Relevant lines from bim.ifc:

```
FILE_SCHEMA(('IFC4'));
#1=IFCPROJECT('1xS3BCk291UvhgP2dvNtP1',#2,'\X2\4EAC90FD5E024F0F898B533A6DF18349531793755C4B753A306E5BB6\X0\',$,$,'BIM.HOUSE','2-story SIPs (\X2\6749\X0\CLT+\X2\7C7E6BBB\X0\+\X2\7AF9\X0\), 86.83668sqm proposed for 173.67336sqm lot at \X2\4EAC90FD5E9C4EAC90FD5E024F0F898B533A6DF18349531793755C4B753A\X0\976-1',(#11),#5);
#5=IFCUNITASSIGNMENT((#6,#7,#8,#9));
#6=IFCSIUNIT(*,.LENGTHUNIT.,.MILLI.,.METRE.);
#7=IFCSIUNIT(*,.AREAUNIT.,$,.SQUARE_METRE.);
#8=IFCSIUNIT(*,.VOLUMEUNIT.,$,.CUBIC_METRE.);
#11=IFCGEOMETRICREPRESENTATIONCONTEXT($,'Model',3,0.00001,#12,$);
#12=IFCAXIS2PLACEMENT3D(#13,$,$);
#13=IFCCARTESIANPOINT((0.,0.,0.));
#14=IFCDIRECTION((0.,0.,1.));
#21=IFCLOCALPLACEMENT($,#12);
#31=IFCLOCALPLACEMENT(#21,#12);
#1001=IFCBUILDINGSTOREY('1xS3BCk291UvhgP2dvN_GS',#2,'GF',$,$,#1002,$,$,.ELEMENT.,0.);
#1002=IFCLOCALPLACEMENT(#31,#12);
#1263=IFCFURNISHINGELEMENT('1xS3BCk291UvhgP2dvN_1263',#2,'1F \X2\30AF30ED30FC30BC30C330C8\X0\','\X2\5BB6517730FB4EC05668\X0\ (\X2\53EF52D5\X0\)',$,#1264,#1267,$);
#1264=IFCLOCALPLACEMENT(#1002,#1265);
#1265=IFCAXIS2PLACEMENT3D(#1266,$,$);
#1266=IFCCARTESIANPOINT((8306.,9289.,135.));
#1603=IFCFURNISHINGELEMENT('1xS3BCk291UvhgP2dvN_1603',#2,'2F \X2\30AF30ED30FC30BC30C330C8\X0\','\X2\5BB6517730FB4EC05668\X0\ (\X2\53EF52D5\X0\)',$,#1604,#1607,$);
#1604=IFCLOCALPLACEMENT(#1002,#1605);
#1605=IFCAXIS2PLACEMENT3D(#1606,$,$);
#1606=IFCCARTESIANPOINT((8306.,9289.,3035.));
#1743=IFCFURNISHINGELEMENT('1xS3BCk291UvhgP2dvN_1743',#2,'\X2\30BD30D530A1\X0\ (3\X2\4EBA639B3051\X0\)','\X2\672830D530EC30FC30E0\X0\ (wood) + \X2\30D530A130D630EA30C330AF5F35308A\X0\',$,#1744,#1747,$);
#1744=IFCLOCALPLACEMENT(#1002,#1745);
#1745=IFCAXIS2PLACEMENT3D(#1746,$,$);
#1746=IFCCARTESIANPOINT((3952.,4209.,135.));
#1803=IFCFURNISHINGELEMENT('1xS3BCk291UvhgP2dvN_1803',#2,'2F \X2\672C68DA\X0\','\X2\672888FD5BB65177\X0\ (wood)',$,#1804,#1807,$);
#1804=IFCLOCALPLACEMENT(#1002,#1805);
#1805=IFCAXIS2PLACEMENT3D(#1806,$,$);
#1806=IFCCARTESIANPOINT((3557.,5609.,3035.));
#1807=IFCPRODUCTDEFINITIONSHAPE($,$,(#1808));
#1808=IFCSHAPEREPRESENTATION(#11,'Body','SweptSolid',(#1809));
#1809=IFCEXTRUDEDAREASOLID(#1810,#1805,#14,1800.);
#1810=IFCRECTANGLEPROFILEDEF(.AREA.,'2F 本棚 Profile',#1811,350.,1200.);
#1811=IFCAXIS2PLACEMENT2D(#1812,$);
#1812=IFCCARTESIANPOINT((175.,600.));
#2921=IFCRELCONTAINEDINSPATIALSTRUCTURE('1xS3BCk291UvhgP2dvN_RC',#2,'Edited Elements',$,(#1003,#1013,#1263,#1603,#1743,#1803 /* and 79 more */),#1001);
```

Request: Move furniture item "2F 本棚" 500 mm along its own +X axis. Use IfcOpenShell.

```python
import ifcopenshell
import ifcopenshell.api.geometry
import ifcopenshell.util.placement

model = ifcopenshell.open("bim.ifc")

item = model.by_guid("1xS3BCk291UvhgP2dvN_1803")
matrix = ifcopenshell.util.placement.get_local_placement(item.ObjectPlacement)
matrix[:3, 3] += matrix[:3, 0] * 500.0
ifcopenshell.api.geometry.edit_object_placement(model, product=item, matrix=matrix, is_si=False)

print(ifcopenshell.util.placement.get_local_placement(item.ObjectPlacement).round(3) + 0.0)

model.write("bim_edited.ifc")
```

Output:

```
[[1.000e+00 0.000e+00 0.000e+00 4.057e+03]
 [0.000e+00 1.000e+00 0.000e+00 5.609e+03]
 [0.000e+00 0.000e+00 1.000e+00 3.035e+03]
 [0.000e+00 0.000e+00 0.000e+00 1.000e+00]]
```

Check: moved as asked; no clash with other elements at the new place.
